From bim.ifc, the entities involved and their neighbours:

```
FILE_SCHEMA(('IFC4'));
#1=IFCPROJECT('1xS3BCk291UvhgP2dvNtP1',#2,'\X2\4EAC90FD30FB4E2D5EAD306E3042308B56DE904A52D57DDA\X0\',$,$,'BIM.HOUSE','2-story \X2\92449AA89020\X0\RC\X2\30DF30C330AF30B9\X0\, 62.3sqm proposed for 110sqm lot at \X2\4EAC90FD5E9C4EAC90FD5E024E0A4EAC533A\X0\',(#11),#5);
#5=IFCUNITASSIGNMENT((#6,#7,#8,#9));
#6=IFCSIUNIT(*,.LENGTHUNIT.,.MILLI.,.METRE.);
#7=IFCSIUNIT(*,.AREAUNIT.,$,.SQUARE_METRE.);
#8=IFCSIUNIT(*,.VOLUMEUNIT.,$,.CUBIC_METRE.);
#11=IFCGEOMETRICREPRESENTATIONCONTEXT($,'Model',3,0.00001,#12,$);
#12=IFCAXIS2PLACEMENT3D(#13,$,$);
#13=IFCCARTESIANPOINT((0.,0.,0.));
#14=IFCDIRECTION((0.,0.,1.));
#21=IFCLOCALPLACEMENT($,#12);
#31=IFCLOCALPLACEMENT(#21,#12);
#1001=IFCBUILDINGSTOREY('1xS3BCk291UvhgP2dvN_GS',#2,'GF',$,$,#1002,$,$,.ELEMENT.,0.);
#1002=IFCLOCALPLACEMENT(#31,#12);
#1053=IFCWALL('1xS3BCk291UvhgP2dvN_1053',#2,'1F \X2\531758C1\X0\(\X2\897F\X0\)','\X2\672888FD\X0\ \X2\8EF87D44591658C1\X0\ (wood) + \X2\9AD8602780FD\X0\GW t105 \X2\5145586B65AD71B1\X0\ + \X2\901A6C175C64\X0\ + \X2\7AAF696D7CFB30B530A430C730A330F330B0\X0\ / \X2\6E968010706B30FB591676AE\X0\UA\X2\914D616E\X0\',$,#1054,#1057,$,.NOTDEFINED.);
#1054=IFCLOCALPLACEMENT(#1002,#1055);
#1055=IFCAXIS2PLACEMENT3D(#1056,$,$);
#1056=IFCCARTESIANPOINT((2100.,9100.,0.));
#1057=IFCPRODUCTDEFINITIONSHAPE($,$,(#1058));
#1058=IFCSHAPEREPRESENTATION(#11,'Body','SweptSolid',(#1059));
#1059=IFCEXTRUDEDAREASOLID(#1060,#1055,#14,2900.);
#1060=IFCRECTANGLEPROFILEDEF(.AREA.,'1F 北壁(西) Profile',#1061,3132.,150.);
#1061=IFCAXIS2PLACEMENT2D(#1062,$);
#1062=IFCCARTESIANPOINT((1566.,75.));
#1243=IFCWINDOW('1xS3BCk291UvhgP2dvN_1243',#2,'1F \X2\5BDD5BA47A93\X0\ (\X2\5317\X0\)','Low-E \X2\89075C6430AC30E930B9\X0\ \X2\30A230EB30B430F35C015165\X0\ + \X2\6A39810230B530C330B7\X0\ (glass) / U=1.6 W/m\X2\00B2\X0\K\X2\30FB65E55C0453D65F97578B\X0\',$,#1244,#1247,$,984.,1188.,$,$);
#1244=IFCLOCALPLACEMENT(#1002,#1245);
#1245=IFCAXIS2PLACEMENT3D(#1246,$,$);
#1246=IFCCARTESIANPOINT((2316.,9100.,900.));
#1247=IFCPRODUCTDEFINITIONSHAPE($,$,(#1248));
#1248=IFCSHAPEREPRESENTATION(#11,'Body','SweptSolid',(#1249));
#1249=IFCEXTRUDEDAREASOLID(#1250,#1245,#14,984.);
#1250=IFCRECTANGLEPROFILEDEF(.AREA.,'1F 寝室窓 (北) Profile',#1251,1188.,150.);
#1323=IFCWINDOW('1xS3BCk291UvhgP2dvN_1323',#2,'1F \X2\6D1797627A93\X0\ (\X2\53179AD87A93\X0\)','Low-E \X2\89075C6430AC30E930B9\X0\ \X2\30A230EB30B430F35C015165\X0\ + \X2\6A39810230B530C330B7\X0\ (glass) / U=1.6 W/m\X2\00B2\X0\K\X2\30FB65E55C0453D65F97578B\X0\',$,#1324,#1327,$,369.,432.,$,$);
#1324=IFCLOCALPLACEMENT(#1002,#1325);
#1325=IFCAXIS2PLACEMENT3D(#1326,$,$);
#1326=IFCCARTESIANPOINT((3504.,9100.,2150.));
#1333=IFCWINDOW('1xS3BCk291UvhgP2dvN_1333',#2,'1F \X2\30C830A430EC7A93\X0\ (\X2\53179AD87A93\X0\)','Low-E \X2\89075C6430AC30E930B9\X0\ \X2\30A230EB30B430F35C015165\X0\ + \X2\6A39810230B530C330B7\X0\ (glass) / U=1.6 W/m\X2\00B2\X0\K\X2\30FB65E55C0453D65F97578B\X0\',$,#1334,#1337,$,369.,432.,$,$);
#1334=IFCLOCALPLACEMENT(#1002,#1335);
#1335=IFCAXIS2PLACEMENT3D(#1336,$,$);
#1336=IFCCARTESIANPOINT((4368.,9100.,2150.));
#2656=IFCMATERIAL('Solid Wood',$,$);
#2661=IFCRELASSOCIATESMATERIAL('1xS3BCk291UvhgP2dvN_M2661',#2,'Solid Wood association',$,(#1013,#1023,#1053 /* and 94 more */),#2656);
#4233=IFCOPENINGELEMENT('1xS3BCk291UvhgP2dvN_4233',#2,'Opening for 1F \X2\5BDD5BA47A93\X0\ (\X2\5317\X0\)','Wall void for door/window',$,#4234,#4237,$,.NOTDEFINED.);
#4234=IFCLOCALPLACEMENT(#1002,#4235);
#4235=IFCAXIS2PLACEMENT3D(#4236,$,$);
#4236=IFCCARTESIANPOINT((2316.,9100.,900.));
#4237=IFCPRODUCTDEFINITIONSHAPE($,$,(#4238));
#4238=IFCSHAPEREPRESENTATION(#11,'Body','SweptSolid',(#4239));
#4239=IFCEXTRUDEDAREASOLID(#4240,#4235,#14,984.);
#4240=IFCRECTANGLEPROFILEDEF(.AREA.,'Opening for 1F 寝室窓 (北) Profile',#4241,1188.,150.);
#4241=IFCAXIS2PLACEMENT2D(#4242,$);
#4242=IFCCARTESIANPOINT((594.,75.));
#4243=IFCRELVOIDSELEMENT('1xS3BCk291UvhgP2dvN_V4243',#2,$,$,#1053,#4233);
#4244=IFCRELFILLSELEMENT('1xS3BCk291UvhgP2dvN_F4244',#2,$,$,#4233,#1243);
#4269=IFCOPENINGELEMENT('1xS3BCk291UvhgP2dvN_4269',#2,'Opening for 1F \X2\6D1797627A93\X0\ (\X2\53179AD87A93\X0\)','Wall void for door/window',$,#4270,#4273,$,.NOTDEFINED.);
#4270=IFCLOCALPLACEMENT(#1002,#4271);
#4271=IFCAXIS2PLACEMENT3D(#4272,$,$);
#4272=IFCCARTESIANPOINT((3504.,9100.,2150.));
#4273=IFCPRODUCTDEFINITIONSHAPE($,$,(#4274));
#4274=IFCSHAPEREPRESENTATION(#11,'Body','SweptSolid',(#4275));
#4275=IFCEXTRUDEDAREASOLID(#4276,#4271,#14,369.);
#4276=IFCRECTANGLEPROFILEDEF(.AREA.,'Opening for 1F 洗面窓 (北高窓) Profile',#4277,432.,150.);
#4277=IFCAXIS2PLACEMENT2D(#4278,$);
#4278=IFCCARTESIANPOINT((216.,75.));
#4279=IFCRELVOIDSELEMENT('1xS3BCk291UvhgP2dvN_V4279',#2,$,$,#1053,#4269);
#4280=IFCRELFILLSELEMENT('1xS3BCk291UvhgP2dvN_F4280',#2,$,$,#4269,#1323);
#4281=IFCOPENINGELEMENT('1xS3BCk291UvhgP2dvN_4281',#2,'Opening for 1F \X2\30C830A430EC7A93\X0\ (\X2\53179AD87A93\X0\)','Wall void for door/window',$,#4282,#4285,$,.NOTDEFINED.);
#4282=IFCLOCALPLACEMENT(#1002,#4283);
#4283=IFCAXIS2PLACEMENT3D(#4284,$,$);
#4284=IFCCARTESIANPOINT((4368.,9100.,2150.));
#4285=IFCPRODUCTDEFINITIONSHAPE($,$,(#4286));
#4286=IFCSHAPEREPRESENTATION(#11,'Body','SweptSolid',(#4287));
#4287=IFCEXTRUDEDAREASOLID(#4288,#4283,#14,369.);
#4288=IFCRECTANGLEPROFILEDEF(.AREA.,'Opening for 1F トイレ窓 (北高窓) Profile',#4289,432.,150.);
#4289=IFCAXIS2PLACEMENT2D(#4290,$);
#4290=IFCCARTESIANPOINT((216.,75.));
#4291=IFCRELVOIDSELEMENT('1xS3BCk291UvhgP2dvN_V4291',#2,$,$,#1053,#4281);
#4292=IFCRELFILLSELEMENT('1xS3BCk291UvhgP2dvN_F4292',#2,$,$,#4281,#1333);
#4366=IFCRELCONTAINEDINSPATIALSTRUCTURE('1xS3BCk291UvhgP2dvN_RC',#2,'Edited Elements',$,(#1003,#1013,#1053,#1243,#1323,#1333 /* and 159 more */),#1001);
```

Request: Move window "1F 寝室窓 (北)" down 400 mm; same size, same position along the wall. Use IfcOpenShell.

```python
import numpy as np
import ifcopenshell
import ifcopenshell.api.geometry
import ifcopenshell.util.placement
import ifcopenshell.util.unit

model = ifcopenshell.open("bim.ifc")
unit_scale = ifcopenshell.util.unit.calculate_unit_scale(model)

window = model.by_guid("1xS3BCk291UvhgP2dvN_1243")
opening = window.FillsVoids[0].RelatingOpeningElement
dz = -0.4 / unit_scale

shift = np.array([0.0, 0.0, dz])
# The window is not placed relative to its opening, so move both.
for product in (opening, window):
    matrix = ifcopenshell.util.placement.get_local_placement(product.ObjectPlacement)
    matrix[:3, 3] += shift
    ifcopenshell.api.geometry.edit_object_placement(model, product=product, matrix=matrix, is_si=False)

print(f"moved by {dz * unit_scale:+.3f} m")

model.write("bim-out.ifc")
```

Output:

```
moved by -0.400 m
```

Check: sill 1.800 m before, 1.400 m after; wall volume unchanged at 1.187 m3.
